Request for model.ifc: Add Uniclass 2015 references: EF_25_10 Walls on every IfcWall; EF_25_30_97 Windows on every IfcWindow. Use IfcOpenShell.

First a look at what the model holds.

```python
import ifcopenshell

model = ifcopenshell.open("model.ifc")
print(model.schema)
print("classifications:", [c.Name for c in model.by_type("IfcClassification")])
for ifc_class in ("IfcDoor", "IfcRoof", "IfcStair", "IfcWall", "IfcWindow"):
    print(ifc_class, len(model.by_type(ifc_class)))
```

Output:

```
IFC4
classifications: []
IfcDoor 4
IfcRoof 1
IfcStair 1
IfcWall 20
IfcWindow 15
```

```python
import ifcopenshell
import ifcopenshell.api.classification

model = ifcopenshell.open("model.ifc")

system = ifcopenshell.api.classification.add_classification(model, classification="Uniclass 2015")

codes = {
    "IfcWall": ("EF_25_10", "Walls"),
    "IfcWindow": ("EF_25_30_97", "Windows"),
}
for ifc_class, (code, name) in codes.items():
    products = model.by_type(ifc_class)
    ifcopenshell.api.classification.add_reference(
        model, products=products, classification=system, identification=code, name=name
    )
    print(code, len(products))

model.write("model_updated.ifc")
```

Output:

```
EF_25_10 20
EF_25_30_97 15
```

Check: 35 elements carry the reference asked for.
